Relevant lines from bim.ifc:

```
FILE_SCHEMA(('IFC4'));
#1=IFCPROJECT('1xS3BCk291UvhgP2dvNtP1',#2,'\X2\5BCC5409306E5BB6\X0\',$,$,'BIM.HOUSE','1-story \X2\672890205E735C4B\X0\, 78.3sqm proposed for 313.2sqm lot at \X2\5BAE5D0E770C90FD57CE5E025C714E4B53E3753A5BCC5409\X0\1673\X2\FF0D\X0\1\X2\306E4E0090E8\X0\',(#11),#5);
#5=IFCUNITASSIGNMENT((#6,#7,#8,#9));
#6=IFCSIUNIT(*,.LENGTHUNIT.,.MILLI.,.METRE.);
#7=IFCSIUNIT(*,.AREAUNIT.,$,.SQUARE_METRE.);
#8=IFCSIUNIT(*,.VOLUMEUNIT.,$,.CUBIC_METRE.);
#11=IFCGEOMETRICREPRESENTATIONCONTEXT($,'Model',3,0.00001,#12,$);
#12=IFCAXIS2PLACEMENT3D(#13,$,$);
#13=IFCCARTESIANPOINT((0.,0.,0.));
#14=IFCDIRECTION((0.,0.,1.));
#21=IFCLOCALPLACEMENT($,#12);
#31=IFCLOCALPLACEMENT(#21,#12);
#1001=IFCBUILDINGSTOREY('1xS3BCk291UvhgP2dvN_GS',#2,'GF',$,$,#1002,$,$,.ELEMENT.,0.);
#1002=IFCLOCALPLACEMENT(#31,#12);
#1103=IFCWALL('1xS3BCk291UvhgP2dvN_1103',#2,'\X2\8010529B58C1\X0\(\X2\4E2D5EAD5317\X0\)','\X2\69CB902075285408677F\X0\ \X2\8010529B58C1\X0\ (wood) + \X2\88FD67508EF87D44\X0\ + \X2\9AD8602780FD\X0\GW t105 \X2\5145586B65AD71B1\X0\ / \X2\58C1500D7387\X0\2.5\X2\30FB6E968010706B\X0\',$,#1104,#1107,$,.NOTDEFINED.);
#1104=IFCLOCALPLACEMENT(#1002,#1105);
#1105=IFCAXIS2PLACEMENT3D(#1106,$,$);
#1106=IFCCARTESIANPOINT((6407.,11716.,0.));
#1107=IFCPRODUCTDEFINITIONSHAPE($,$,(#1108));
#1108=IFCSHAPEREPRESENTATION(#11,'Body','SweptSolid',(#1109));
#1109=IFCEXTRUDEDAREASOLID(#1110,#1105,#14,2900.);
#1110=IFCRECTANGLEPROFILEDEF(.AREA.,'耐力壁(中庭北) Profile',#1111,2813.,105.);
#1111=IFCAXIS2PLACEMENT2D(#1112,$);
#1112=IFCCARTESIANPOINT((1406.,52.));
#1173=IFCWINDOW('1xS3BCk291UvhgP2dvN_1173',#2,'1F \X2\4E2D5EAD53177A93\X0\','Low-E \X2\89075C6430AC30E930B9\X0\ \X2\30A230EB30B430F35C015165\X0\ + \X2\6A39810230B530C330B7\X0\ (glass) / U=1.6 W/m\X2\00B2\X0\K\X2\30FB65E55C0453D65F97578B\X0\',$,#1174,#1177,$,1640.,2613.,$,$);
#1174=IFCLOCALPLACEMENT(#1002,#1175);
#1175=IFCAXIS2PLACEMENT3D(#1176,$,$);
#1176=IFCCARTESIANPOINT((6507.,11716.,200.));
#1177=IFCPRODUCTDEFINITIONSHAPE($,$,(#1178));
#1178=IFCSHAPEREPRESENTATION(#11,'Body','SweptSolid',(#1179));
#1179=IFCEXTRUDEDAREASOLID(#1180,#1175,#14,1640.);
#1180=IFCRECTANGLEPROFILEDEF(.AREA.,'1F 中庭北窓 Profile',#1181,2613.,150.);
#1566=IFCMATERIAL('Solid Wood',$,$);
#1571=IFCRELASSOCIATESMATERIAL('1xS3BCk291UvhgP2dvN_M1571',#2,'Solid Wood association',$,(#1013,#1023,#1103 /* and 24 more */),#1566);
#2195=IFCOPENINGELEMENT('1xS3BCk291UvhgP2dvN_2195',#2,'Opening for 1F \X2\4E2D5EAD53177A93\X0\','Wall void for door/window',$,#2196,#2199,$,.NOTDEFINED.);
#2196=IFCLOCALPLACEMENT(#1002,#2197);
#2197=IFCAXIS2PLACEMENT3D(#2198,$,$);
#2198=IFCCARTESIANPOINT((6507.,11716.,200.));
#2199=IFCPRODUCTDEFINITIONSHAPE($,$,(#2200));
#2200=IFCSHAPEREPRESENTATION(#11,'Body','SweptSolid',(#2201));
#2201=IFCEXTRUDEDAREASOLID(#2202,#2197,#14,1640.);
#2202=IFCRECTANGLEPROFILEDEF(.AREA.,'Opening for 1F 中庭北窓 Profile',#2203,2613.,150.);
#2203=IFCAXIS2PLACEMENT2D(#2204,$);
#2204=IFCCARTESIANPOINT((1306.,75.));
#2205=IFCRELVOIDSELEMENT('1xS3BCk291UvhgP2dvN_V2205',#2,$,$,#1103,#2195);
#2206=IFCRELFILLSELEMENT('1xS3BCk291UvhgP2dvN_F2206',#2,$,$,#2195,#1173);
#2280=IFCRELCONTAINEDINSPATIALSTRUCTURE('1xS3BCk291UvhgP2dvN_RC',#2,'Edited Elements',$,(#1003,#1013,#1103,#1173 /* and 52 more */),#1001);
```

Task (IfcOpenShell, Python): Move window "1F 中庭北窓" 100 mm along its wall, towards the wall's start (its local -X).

```python
import ifcopenshell
import ifcopenshell.api.geometry
import ifcopenshell.util.placement

model = ifcopenshell.open("bim.ifc")

window = model.by_guid("1xS3BCk291UvhgP2dvN_1173")
opening = window.FillsVoids[0].RelatingOpeningElement
wall = opening.VoidsElements[0].RelatingBuildingElement

wall_matrix = ifcopenshell.util.placement.get_local_placement(wall.ObjectPlacement)
shift = wall_matrix[:3, 0] * -100.0
before = ifcopenshell.util.placement.get_local_placement(window.ObjectPlacement)[:3, 3].copy()

# The window is not placed relative to its opening, so move both.
for product in (opening, window):
    matrix = ifcopenshell.util.placement.get_local_placement(product.ObjectPlacement)
    matrix[:3, 3] += shift
    ifcopenshell.api.geometry.edit_object_placement(model, product=product, matrix=matrix, is_si=False)

after = ifcopenshell.util.placement.get_local_placement(window.ObjectPlacement)[:3, 3]
print("window moved by", (after - before).round(3) + 0.0)

model.write("bim-out.ifc")
```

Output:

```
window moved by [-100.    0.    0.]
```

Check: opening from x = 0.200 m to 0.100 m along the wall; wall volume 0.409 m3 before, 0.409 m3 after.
